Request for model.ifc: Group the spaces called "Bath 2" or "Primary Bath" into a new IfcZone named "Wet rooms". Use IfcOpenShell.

First a look at what the model holds.

```python
import ifcopenshell

model = ifcopenshell.open("model.ifc")
print(model.schema)
seen = {}
for space in model.by_type("IfcSpace"):
    seen[space.LongName] = seen.get(space.LongName, 0) + 1
for name, count in sorted(seen.items(), key=str):
    print(count, "x", name)
print("zones:", [z.Name for z in model.by_type("IfcZone")][:20])
```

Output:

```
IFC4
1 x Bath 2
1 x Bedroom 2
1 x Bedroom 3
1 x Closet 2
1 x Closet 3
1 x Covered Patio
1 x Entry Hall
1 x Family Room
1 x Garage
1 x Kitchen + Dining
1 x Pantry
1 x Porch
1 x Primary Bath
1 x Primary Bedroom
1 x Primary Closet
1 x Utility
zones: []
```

```python
import ifcopenshell
import ifcopenshell.api.group
import ifcopenshell.api.root

model = ifcopenshell.open("model.ifc")

names = {"Bath 2", "Primary Bath"}
spaces = [s for s in model.by_type("IfcSpace") if s.LongName in names]

zone = ifcopenshell.api.root.create_entity(model, ifc_class="IfcZone", name="Wet rooms")
ifcopenshell.api.group.assign_group(model, products=spaces, group=zone)
print(len(spaces), "spaces in", zone.Name)

model.write("model-out.ifc")
```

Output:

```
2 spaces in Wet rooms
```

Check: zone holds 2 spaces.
